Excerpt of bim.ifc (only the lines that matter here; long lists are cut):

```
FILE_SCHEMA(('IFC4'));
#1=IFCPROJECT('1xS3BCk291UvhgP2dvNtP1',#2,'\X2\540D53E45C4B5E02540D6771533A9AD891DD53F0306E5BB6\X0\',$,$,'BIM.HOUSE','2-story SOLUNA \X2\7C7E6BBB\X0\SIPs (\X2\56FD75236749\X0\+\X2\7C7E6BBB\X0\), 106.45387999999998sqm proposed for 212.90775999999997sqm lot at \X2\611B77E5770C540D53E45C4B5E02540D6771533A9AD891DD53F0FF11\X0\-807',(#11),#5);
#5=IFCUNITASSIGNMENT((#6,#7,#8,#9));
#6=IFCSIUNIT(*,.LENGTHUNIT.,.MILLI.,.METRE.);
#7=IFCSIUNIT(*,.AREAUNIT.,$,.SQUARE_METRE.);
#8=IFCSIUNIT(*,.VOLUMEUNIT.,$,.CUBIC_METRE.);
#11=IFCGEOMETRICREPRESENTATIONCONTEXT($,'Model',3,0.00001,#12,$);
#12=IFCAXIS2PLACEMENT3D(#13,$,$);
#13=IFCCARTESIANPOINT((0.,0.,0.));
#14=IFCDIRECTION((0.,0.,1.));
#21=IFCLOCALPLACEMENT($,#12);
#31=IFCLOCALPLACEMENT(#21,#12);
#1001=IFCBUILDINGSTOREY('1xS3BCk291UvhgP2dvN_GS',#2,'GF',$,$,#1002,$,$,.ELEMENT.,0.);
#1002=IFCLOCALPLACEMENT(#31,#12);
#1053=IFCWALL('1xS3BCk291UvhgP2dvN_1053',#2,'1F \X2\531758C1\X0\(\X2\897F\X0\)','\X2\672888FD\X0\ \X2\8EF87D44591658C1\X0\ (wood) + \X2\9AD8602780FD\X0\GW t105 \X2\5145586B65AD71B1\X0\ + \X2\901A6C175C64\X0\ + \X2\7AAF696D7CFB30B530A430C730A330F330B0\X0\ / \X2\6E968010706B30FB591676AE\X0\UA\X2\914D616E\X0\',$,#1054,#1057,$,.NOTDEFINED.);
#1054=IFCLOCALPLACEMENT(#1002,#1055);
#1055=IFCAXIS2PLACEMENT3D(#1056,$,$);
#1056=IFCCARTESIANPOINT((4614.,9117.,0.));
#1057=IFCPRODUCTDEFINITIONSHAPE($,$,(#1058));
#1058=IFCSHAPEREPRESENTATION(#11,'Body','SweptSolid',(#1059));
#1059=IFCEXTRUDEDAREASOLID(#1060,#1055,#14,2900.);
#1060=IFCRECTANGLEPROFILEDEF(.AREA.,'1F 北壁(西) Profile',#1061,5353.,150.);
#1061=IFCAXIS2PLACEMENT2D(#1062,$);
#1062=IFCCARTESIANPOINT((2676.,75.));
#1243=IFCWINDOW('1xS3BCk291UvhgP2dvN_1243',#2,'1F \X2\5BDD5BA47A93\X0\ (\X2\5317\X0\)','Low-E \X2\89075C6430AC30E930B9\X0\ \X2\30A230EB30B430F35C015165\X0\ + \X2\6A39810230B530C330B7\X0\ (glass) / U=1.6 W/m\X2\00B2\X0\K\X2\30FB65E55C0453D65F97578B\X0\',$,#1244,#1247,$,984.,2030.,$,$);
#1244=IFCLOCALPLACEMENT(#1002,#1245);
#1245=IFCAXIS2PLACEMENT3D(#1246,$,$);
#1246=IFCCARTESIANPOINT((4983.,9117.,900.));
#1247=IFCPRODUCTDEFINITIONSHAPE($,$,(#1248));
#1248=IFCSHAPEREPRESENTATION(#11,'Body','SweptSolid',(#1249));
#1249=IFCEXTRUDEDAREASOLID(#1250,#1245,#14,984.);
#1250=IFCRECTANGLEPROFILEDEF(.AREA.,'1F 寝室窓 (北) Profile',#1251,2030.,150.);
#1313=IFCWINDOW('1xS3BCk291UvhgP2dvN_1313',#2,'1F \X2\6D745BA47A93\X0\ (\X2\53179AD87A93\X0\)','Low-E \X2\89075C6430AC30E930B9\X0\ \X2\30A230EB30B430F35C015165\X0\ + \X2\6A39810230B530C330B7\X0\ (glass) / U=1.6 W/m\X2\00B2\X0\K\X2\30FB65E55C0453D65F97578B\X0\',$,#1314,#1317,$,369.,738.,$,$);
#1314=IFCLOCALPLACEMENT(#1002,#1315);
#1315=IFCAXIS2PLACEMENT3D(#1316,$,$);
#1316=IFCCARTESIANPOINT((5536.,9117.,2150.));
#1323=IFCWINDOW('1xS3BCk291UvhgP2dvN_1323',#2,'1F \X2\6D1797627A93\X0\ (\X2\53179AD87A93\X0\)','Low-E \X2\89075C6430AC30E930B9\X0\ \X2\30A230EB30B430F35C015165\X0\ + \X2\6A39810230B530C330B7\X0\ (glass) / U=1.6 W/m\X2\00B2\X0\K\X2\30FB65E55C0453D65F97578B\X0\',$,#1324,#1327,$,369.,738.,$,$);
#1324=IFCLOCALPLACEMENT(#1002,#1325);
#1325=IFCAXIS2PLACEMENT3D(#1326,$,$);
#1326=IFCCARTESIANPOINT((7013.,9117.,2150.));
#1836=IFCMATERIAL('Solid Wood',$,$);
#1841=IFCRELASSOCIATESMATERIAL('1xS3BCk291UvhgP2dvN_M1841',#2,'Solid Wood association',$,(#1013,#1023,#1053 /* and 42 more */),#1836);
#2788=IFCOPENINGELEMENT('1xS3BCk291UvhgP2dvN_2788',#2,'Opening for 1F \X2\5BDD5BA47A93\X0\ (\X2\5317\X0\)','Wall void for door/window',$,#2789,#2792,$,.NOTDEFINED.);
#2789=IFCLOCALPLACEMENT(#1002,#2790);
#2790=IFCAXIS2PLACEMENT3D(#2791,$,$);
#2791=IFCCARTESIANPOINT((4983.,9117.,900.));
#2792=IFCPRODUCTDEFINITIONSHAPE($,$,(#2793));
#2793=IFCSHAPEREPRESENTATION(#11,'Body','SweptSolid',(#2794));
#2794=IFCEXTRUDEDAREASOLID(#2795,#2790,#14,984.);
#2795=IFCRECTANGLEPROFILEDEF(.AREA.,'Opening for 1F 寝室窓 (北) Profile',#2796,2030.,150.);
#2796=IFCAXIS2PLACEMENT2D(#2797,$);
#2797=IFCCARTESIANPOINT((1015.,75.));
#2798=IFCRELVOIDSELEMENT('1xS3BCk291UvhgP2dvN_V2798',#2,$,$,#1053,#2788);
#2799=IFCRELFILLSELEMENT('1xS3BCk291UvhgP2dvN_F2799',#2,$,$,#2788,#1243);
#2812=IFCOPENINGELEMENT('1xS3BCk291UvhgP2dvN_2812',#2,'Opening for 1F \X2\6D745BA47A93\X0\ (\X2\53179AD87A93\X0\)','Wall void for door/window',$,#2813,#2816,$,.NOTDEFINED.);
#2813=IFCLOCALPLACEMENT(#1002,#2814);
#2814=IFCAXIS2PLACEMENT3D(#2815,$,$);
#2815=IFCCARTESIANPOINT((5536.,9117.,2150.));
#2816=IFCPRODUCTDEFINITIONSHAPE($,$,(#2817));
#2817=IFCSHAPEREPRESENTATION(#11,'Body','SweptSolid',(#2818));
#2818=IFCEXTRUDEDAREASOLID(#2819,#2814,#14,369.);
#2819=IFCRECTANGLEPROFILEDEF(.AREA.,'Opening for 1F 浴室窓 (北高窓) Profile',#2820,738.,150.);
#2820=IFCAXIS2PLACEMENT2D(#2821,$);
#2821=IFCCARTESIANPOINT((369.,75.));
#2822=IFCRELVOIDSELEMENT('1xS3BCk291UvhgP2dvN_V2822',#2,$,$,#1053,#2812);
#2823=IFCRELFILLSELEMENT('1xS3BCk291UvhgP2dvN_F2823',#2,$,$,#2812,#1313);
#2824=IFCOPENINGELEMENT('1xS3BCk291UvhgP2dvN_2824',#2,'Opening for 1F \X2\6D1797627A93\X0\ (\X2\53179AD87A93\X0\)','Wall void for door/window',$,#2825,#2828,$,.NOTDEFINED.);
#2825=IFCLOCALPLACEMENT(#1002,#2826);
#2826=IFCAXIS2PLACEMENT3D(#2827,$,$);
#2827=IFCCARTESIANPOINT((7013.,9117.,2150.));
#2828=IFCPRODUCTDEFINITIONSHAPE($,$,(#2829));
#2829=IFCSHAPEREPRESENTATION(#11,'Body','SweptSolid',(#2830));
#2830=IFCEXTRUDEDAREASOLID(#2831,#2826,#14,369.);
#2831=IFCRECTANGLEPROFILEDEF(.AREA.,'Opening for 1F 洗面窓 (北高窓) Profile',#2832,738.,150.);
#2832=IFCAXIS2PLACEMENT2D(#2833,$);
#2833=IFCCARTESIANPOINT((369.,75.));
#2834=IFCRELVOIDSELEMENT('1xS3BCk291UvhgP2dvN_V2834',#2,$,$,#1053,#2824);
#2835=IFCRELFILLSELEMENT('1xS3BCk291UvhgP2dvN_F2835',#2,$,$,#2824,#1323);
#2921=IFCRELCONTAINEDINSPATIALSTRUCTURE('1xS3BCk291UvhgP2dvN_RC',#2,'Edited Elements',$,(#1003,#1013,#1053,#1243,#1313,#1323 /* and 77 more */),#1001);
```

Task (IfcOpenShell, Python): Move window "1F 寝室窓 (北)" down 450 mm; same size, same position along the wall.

```python
import numpy as np
import ifcopenshell
import ifcopenshell.api.geometry
import ifcopenshell.util.placement
import ifcopenshell.util.unit

model = ifcopenshell.open("bim.ifc")
unit_scale = ifcopenshell.util.unit.calculate_unit_scale(model)

window = model.by_guid("1xS3BCk291UvhgP2dvN_1243")
opening = window.FillsVoids[0].RelatingOpeningElement
dz = -450.0

shift = np.array([0.0, 0.0, dz])
# The window is not placed relative to its opening, so move both.
for product in (opening, window):
    matrix = ifcopenshell.util.placement.get_local_placement(product.ObjectPlacement)
    matrix[:3, 3] += shift
    ifcopenshell.api.geometry.edit_object_placement(model, product=product, matrix=matrix, is_si=False)

print(f"moved by {dz * unit_scale:+.3f} m")

model.write("bim_v2.ifc")
```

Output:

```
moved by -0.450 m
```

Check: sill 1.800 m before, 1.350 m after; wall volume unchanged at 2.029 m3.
